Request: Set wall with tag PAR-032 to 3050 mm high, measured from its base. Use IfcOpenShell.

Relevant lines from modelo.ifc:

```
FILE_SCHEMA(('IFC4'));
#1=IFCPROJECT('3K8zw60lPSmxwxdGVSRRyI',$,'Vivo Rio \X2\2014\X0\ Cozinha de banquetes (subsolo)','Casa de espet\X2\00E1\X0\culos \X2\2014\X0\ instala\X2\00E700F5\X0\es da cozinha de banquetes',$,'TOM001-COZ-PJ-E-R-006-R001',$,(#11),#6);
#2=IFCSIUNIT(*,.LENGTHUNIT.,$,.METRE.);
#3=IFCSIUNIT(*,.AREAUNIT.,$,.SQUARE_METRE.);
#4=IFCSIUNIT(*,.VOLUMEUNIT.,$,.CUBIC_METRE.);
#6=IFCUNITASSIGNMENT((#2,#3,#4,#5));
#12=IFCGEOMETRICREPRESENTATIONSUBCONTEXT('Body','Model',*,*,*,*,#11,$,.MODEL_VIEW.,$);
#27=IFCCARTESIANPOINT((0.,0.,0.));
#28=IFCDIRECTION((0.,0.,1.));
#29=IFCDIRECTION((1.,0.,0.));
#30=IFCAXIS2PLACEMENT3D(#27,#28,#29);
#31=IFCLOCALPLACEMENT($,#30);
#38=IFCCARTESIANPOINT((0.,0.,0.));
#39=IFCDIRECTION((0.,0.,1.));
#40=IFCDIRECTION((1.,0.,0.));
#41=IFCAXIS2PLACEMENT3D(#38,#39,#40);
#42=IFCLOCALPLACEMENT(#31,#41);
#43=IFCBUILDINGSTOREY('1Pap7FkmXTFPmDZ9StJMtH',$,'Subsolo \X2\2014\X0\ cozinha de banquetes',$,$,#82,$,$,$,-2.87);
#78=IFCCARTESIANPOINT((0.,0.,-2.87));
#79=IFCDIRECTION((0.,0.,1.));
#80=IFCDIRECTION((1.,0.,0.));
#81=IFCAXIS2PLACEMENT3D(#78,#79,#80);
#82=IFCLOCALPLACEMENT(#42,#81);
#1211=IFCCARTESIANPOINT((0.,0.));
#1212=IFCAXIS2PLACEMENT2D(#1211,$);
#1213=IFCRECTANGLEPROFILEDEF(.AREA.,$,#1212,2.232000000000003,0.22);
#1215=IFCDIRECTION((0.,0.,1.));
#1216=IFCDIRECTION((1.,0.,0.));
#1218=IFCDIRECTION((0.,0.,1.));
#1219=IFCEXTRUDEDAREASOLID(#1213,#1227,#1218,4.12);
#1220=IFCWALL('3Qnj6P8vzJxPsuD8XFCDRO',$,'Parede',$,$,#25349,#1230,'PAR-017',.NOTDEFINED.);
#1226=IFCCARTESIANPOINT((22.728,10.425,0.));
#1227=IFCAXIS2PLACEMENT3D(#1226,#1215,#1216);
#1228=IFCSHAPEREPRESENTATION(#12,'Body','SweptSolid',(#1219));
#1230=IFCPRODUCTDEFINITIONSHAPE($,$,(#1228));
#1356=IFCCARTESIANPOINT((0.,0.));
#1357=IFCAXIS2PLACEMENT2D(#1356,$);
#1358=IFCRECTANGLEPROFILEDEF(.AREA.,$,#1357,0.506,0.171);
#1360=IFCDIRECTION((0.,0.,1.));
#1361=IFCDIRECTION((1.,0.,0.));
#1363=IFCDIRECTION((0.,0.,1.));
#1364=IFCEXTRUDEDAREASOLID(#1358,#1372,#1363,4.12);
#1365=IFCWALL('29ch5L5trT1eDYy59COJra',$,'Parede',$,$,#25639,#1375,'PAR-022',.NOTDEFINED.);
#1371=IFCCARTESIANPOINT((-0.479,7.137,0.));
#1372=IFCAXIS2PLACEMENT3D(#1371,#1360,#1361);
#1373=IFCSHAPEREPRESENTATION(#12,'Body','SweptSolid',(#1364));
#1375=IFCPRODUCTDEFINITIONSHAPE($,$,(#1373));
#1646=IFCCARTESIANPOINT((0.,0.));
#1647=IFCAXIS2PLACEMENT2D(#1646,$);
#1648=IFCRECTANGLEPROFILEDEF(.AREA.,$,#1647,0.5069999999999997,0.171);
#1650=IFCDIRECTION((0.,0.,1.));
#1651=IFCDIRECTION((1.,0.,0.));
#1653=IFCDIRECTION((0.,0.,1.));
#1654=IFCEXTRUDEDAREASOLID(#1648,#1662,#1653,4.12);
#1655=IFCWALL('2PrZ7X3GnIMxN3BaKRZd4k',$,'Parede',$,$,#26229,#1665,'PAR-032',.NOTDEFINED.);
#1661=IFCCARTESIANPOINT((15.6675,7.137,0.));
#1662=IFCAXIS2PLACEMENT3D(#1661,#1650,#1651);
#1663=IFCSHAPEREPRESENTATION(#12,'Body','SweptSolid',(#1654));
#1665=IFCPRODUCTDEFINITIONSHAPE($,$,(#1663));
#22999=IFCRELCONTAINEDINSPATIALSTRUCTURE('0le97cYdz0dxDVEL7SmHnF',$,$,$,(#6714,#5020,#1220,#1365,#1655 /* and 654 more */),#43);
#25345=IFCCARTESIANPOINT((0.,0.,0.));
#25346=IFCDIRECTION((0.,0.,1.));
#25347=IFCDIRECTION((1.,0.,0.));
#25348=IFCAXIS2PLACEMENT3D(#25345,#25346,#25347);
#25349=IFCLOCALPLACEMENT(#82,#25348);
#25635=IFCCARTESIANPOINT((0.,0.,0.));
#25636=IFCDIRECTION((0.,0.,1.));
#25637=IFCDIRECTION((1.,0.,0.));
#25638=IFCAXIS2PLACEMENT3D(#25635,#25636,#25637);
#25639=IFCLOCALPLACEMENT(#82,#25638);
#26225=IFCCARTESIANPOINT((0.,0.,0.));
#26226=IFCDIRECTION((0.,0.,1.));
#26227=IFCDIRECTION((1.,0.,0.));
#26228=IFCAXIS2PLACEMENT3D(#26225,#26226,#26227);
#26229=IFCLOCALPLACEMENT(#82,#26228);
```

```python
import ifcopenshell
import ifcopenshell.geom
import ifcopenshell.util.representation
import ifcopenshell.util.shape
import ifcopenshell.util.unit

model = ifcopenshell.open("modelo.ifc")
unit_scale = ifcopenshell.util.unit.calculate_unit_scale(model)
settings = ifcopenshell.geom.settings()


def volume(element):
    """Net volume in cubic metres, openings subtracted."""
    shape = ifcopenshell.geom.create_shape(settings, element)
    return ifcopenshell.util.shape.get_volume(shape.geometry)


wall = model.by_id(1655)
before = volume(wall)

body = ifcopenshell.util.representation.get_representation(wall, "Model", "Body")
solid = body.Items[0]
old_height = solid.Depth
solid.Depth = 3.05 / unit_scale
after = volume(wall)

print(f"height {old_height:g} -> {solid.Depth:g}, volume {before:.3f} -> {after:.3f} m3")

model.write("modelo_edited.ifc")
```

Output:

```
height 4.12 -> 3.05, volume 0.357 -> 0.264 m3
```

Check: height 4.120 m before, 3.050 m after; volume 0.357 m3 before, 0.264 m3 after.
